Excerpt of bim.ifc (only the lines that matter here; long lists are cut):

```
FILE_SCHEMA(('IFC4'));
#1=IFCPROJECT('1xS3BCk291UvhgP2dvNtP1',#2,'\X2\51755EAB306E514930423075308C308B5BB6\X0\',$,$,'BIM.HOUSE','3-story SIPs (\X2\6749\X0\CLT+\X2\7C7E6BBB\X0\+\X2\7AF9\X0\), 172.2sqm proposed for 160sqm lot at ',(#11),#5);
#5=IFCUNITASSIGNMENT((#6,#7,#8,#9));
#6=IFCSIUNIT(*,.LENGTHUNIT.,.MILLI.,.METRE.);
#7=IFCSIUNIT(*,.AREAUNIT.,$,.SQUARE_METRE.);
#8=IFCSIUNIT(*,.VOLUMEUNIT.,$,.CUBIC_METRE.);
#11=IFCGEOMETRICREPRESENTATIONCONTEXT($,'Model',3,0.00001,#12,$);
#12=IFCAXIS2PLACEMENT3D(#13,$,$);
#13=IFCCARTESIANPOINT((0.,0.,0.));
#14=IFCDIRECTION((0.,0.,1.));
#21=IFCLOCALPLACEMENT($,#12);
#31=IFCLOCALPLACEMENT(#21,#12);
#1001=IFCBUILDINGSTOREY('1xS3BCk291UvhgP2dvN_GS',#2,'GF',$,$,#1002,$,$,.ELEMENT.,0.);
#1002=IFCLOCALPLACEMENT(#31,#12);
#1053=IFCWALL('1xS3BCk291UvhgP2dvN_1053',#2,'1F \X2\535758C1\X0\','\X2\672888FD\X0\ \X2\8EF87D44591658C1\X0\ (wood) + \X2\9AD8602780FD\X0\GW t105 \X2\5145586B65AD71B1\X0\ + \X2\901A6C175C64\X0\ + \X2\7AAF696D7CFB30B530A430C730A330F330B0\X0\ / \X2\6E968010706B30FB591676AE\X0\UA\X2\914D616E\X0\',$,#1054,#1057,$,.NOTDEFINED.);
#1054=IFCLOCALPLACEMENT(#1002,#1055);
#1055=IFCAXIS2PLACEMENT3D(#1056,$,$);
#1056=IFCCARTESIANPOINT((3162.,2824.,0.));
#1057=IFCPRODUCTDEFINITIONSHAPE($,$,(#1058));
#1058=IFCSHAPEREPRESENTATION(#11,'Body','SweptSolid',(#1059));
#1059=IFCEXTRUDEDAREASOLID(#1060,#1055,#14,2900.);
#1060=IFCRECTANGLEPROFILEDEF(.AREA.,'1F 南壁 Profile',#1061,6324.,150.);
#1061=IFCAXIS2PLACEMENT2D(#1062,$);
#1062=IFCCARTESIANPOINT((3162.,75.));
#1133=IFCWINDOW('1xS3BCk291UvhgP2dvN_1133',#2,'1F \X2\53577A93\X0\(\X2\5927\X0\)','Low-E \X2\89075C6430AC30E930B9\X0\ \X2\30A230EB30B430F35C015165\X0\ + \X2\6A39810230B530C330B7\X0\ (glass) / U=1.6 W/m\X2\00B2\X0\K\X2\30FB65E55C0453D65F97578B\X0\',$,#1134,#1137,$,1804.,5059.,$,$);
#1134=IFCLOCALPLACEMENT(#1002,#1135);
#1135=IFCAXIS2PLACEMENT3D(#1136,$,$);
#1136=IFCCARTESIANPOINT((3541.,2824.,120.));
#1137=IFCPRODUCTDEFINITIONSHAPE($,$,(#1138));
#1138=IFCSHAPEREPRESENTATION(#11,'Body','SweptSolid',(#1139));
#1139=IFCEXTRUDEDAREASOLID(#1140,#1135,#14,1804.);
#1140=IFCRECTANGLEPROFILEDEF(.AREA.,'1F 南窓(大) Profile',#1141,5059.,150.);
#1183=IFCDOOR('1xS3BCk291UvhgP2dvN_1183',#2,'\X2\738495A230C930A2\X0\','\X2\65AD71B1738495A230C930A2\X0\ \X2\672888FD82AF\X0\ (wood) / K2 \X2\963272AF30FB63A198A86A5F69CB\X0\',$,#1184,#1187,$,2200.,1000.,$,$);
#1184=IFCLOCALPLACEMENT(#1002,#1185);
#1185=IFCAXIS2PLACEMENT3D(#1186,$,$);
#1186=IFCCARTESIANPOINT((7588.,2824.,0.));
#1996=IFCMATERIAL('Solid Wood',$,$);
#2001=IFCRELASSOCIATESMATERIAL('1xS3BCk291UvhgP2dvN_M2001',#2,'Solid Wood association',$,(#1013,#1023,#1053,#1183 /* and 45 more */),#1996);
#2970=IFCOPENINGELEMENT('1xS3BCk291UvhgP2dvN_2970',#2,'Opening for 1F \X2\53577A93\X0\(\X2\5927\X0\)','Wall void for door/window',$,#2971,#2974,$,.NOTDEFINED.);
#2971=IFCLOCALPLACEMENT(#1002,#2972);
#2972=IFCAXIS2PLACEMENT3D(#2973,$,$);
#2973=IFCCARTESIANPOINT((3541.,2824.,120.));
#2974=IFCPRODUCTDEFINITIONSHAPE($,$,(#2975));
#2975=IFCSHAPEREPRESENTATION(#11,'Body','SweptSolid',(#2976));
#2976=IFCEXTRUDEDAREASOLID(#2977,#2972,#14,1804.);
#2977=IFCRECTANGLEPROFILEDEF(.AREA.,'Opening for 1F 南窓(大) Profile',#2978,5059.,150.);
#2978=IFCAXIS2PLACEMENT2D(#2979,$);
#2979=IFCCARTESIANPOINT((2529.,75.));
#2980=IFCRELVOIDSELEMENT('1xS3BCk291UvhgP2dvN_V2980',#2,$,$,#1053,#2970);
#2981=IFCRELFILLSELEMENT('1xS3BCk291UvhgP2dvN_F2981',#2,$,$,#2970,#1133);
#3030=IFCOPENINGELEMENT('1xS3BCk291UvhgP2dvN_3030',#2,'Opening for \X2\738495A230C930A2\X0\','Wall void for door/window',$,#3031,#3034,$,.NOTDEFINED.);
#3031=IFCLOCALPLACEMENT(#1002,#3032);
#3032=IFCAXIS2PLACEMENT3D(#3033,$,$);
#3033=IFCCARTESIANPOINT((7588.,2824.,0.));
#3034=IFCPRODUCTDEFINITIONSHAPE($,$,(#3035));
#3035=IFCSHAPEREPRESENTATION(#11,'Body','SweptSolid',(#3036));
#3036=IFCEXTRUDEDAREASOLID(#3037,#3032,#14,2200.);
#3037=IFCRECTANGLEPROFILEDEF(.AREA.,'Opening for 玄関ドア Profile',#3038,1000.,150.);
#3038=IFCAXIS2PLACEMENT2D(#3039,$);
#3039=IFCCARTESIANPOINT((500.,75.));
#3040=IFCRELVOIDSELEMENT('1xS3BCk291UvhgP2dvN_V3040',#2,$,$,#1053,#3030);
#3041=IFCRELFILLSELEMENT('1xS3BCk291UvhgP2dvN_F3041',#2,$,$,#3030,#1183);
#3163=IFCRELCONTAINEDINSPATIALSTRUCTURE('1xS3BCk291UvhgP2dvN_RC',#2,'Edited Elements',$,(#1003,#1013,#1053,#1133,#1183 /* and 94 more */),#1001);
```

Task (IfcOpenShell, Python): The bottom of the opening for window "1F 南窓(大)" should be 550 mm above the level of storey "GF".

```python
import numpy as np
import ifcopenshell
import ifcopenshell.api.geometry
import ifcopenshell.geom
import ifcopenshell.util.element
import ifcopenshell.util.placement
import ifcopenshell.util.shape
import ifcopenshell.util.unit

model = ifcopenshell.open("bim.ifc")
unit_scale = ifcopenshell.util.unit.calculate_unit_scale(model)

window = model.by_id(1133)
opening = window.FillsVoids[0].RelatingOpeningElement
storey = ifcopenshell.util.element.get_container(window, ifc_class="IfcBuildingStorey")
level = ifcopenshell.util.placement.get_local_placement(storey.ObjectPlacement)[2, 3]

# The opening's origin need not be at the sill, so measure its lowest point.
shape = ifcopenshell.geom.create_shape(ifcopenshell.geom.settings(), opening)
bottom = ifcopenshell.util.shape.get_shape_bottom_elevation(shape, shape.geometry) / unit_scale
dz = level + 550.0 - bottom

shift = np.array([0.0, 0.0, dz])
# The window is not placed relative to its opening, so move both.
for product in (opening, window):
    matrix = ifcopenshell.util.placement.get_local_placement(product.ObjectPlacement)
    matrix[:3, 3] += shift
    ifcopenshell.api.geometry.edit_object_placement(model, product=product, matrix=matrix, is_si=False)

print(f"moved by {dz * unit_scale:+.3f} m")

model.write("bim_rev.ifc")
```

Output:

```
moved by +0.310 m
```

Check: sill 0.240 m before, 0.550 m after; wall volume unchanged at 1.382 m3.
